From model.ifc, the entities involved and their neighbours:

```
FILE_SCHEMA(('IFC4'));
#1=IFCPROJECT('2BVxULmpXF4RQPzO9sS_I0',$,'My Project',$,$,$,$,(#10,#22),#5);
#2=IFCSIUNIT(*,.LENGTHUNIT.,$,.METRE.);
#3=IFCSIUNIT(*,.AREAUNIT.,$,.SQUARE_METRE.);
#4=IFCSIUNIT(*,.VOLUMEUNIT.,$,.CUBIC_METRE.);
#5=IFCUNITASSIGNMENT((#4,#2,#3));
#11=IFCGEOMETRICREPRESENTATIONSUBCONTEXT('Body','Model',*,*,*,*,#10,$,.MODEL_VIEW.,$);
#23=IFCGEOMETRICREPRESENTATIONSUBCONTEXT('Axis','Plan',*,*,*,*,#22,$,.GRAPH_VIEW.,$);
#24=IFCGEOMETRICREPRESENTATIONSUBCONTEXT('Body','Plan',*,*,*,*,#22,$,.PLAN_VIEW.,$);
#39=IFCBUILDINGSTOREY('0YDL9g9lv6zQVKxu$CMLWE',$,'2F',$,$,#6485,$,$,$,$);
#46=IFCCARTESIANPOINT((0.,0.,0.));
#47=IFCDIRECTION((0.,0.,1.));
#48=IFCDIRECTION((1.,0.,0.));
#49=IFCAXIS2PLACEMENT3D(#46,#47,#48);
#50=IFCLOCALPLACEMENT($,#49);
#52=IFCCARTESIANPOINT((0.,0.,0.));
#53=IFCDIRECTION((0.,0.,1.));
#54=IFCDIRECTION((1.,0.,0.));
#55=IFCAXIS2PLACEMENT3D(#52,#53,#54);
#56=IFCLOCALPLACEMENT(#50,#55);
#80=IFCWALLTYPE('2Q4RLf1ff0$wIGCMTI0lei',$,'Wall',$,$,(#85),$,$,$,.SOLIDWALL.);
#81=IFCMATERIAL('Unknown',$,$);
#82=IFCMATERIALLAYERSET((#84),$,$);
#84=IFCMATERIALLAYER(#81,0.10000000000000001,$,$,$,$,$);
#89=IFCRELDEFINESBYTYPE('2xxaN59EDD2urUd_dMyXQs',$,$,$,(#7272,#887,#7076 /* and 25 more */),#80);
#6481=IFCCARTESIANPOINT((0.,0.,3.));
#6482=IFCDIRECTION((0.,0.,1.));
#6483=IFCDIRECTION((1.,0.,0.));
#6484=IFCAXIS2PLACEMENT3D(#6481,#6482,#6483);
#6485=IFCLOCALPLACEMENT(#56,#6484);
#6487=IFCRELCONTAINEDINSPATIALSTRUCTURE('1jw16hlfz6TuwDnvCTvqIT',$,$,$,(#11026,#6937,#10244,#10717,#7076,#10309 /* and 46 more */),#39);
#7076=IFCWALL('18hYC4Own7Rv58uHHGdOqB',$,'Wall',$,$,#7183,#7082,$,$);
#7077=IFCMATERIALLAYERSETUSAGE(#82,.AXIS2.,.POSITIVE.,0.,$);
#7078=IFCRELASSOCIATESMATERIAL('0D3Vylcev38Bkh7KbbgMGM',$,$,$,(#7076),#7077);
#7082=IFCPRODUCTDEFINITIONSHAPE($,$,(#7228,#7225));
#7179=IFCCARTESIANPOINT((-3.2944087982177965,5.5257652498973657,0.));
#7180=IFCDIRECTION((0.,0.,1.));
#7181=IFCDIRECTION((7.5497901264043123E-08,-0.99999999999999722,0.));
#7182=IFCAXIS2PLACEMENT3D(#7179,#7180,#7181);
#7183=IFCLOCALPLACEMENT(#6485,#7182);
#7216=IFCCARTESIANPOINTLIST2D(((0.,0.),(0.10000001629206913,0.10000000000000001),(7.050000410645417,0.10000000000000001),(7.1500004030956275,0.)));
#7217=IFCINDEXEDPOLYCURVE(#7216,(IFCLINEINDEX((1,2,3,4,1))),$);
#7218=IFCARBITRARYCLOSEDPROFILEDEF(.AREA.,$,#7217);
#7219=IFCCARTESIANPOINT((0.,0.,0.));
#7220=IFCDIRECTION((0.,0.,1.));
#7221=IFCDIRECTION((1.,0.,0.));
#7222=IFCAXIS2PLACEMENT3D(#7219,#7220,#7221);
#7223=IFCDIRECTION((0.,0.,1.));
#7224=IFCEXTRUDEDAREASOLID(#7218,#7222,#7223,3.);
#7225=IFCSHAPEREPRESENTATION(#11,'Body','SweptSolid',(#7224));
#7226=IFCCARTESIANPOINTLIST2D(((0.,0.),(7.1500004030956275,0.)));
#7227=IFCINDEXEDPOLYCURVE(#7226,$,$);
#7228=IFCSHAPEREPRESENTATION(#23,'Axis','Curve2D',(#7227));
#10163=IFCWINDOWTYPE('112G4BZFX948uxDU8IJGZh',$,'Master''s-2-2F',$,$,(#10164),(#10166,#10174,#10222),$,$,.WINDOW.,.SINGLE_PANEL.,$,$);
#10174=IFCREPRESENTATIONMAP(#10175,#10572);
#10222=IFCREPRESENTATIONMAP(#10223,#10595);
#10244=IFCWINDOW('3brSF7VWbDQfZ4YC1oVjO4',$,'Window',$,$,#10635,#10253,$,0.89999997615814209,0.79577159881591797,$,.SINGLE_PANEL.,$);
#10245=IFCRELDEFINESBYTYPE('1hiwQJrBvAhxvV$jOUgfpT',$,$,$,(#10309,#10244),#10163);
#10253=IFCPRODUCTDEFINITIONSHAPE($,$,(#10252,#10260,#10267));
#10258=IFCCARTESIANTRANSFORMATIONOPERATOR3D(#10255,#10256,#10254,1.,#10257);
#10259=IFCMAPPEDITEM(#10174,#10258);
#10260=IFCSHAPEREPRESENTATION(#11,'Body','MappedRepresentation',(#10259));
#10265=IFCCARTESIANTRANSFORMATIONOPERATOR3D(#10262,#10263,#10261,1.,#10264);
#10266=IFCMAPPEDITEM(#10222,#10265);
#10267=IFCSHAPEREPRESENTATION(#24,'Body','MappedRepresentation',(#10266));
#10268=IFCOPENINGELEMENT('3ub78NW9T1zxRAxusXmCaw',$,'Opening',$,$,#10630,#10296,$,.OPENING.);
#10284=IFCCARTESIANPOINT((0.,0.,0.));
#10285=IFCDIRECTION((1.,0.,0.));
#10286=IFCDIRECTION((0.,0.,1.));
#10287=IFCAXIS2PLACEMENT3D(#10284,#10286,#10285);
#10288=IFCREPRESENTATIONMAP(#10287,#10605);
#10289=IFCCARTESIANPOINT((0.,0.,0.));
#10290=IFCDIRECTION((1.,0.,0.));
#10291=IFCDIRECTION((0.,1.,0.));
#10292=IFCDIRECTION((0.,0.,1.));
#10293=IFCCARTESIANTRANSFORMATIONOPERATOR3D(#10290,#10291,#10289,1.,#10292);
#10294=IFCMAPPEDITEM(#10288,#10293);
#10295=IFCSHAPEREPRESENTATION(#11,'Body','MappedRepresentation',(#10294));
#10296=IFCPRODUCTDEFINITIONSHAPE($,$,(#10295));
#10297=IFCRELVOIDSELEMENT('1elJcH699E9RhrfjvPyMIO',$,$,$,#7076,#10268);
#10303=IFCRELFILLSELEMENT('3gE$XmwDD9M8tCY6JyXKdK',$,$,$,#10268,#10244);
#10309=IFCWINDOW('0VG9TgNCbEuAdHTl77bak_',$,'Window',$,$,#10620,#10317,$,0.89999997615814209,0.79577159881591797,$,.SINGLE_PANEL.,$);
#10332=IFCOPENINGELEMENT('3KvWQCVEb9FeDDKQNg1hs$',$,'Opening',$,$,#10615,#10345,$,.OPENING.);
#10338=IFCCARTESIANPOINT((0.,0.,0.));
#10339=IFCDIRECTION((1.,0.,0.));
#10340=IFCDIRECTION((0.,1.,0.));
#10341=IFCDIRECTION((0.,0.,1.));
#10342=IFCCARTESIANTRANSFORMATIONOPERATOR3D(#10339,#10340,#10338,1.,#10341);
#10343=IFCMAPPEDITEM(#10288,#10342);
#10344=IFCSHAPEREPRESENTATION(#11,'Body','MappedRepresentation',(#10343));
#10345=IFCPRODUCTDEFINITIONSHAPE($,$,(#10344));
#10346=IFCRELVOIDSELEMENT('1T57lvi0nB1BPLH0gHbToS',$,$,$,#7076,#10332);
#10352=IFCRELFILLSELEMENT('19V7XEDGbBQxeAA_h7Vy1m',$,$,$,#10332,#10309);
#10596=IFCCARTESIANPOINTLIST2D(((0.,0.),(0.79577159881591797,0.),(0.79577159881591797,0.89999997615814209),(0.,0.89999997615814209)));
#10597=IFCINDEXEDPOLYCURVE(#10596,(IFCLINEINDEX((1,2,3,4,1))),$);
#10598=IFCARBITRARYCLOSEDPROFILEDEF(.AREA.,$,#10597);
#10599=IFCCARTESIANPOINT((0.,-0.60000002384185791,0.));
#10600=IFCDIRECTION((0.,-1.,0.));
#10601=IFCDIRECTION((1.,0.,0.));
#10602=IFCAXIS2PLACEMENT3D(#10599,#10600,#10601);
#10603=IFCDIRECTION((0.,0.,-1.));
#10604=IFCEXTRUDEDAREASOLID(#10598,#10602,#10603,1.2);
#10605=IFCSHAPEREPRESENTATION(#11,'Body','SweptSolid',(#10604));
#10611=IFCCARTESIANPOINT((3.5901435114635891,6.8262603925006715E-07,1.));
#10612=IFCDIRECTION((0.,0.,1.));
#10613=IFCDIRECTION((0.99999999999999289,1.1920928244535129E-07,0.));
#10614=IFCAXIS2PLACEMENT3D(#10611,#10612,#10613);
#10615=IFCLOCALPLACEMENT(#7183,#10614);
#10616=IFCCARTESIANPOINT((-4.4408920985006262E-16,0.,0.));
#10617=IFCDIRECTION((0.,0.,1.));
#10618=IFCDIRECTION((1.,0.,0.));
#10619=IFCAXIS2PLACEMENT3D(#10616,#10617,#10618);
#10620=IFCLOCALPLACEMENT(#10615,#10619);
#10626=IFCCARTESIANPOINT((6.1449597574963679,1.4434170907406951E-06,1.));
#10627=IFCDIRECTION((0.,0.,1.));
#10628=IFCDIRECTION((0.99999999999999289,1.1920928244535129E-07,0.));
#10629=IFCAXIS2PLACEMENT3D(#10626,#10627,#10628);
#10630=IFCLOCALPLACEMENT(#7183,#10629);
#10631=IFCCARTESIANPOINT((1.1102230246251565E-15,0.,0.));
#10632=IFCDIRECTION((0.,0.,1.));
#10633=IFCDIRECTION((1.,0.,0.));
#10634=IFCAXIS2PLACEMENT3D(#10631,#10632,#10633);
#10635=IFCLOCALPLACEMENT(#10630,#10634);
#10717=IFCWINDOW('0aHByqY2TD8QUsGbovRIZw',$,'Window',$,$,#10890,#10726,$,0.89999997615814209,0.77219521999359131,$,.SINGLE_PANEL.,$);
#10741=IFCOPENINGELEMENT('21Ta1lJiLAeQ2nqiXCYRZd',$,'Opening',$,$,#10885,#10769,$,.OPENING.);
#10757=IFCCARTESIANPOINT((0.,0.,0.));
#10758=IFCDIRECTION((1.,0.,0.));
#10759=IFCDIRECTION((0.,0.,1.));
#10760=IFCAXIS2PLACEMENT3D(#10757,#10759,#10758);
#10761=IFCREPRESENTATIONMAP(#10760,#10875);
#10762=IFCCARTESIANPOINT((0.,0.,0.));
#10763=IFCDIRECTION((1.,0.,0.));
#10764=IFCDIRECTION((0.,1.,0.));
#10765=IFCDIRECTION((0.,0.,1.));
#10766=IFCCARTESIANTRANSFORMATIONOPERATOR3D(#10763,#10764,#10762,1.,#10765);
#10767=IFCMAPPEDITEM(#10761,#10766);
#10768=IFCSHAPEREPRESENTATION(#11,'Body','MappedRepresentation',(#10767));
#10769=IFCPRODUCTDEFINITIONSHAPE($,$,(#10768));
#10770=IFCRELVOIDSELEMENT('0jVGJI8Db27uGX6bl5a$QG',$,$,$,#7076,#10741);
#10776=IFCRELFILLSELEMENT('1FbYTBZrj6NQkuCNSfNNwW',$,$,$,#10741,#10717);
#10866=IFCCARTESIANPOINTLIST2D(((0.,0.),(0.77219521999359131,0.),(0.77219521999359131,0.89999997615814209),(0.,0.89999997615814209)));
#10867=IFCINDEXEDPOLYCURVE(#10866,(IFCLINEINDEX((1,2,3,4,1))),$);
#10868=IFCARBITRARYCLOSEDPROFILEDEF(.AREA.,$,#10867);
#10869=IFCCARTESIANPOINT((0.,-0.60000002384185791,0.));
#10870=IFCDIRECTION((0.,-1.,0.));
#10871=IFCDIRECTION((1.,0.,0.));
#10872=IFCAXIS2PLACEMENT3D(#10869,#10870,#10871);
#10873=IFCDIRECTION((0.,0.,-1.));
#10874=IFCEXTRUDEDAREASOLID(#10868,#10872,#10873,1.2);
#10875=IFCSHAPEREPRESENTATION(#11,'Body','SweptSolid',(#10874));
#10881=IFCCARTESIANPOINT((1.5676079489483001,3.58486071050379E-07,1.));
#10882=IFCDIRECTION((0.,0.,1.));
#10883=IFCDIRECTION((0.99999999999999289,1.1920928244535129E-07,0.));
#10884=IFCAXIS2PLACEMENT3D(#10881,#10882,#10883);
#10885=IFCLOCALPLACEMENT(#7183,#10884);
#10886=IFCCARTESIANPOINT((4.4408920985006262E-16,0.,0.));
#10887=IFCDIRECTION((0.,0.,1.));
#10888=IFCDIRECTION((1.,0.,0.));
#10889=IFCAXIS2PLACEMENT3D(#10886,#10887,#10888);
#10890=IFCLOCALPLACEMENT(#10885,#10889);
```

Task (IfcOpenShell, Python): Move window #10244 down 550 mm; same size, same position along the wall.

```python
import numpy as np
import ifcopenshell
import ifcopenshell.api.geometry
import ifcopenshell.util.placement
import ifcopenshell.util.unit

model = ifcopenshell.open("model.ifc")
unit_scale = ifcopenshell.util.unit.calculate_unit_scale(model)

window = model.by_id(10244)
opening = window.FillsVoids[0].RelatingOpeningElement
dz = -0.55

shift = np.array([0.0, 0.0, dz])
# The window is placed relative to its opening, so it follows when the opening moves.
matrix = ifcopenshell.util.placement.get_local_placement(opening.ObjectPlacement)
matrix[:3, 3] += shift
ifcopenshell.api.geometry.edit_object_placement(
    model, product=opening, matrix=matrix, is_si=False, should_transform_children=True
)

print(f"moved by {dz * unit_scale:+.3f} m")

model.write("model_v2.ifc")
```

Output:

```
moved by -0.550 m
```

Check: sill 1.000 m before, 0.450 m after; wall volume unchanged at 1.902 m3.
